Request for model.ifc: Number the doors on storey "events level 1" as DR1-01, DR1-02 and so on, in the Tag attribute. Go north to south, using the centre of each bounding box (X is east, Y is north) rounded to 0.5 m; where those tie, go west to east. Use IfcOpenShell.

First a look at what the model holds.

```python
import ifcopenshell
import ifcopenshell.util.element
import ifcopenshell.util.placement

model = ifcopenshell.open("model.ifc")
print(model.schema)
storey = next(s for s in model.by_type("IfcBuildingStorey") if s.Name == "events level 1")
doors = [e for e in ifcopenshell.util.element.get_decomposition(storey) if e.is_a("IfcDoor")]
for e in sorted(doors, key=lambda e: e.id()):
    origin = ifcopenshell.util.placement.get_local_placement(e.ObjectPlacement)[:3, 3]
    print(e.id(), e.Tag, e.Name, origin.round(2) + 0.0, sep=" | ")
```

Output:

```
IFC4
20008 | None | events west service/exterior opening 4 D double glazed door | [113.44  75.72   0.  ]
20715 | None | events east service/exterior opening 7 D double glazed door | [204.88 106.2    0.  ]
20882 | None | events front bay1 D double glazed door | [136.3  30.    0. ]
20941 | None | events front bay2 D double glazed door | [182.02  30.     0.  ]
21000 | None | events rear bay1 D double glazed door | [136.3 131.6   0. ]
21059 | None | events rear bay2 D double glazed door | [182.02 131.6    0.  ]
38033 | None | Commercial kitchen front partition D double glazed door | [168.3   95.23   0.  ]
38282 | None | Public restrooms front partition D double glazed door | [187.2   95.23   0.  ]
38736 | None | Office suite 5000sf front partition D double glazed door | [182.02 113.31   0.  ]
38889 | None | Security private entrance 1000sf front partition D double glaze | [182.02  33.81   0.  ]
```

```python
import ifcopenshell
import ifcopenshell.geom
import ifcopenshell.util.element
import ifcopenshell.util.shape

model = ifcopenshell.open("model.ifc")
settings = ifcopenshell.geom.settings()
settings.set("use-world-coords", True)


def centre(element):
    shape = ifcopenshell.geom.create_shape(settings, element)
    return ifcopenshell.util.shape.get_bbox_centroid(shape.geometry)


storey = next(s for s in model.by_type("IfcBuildingStorey") if s.Name == "events level 1")
doors = [e for e in ifcopenshell.util.element.get_decomposition(storey) if e.is_a("IfcDoor")]

# Insertion points can sit at a corner or the storey origin, so sort by the geometry (in metres).
centres = {e: centre(e) for e in doors}
doors.sort(key=lambda e: (-round(centres[e][1] / 0.5), centres[e][0]))

for i, e in enumerate(doors, start=1):
    number = f"DR1-{i:02d}"
    e.Tag = number
    print(e.id(), number)

model.write("model_v2.ifc")
```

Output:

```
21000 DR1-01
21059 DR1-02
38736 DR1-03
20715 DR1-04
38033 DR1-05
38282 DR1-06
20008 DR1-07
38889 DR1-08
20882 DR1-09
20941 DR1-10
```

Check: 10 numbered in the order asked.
